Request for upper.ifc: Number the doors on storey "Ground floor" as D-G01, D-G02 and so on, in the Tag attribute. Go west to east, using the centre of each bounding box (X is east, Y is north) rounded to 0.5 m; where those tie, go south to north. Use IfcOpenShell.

First a look at what the model holds.

```python
import ifcopenshell
import ifcopenshell.util.element
import ifcopenshell.util.placement

model = ifcopenshell.open("upper.ifc")
print(model.schema)
storey = next(s for s in model.by_type("IfcBuildingStorey") if s.Name == "Ground floor")
doors = [e for e in ifcopenshell.util.element.get_decomposition(storey) if e.is_a("IfcDoor")]
for e in sorted(doors, key=lambda e: e.id()):
    origin = ifcopenshell.util.placement.get_local_placement(e.ObjectPlacement)[:3, 3]
    print(e.id(), e.Tag, e.Name, origin.round(2) + 0.0, sep=" | ")
```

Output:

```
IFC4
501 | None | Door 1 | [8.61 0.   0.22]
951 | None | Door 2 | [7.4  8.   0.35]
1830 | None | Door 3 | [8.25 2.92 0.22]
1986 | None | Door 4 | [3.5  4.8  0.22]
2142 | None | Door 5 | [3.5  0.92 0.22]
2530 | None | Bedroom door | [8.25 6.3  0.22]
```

```python
import ifcopenshell
import ifcopenshell.geom
import ifcopenshell.util.element
import ifcopenshell.util.shape

model = ifcopenshell.open("upper.ifc")
settings = ifcopenshell.geom.settings()
settings.set("use-world-coords", True)


def centre(element):
    shape = ifcopenshell.geom.create_shape(settings, element)
    return ifcopenshell.util.shape.get_bbox_centroid(shape.geometry)


storey = next(s for s in model.by_type("IfcBuildingStorey") if s.Name == "Ground floor")
doors = [e for e in ifcopenshell.util.element.get_decomposition(storey) if e.is_a("IfcDoor")]

# Insertion points can sit at a corner or the storey origin, so sort by the geometry (in metres).
centres = {e: centre(e) for e in doors}
doors.sort(key=lambda e: (round(centres[e][0] / 0.5), centres[e][1]))

for i, e in enumerate(doors, start=1):
    number = f"D-G{i:02d}"
    e.Tag = number
    print(e.id(), number)

model.write("upper-out.ifc")
```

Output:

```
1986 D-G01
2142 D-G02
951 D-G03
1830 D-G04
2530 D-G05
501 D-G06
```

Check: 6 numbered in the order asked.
